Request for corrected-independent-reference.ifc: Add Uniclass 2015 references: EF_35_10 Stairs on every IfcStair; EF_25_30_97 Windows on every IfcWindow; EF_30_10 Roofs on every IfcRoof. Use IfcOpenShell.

First a look at what the model holds.

```python
import ifcopenshell

model = ifcopenshell.open("corrected-independent-reference.ifc")
print(model.schema)
print("classifications:", [c.Name for c in model.by_type("IfcClassification")])
for ifc_class in ("IfcDoor", "IfcRoof", "IfcStair", "IfcWall", "IfcWindow"):
    print(ifc_class, len(model.by_type(ifc_class)))
```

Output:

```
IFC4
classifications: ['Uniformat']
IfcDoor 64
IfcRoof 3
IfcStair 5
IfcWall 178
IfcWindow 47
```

```python
import ifcopenshell
import ifcopenshell.api.classification

model = ifcopenshell.open("corrected-independent-reference.ifc")

system = ifcopenshell.api.classification.add_classification(model, classification="Uniclass 2015")

codes = {
    "IfcStair": ("EF_35_10", "Stairs"),
    "IfcWindow": ("EF_25_30_97", "Windows"),
    "IfcRoof": ("EF_30_10", "Roofs"),
}
for ifc_class, (code, name) in codes.items():
    products = model.by_type(ifc_class)
    ifcopenshell.api.classification.add_reference(
        model, products=products, classification=system, identification=code, name=name
    )
    print(code, len(products))

model.write("corrected-independent-reference-out.ifc")
```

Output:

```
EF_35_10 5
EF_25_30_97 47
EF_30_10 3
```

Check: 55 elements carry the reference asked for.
